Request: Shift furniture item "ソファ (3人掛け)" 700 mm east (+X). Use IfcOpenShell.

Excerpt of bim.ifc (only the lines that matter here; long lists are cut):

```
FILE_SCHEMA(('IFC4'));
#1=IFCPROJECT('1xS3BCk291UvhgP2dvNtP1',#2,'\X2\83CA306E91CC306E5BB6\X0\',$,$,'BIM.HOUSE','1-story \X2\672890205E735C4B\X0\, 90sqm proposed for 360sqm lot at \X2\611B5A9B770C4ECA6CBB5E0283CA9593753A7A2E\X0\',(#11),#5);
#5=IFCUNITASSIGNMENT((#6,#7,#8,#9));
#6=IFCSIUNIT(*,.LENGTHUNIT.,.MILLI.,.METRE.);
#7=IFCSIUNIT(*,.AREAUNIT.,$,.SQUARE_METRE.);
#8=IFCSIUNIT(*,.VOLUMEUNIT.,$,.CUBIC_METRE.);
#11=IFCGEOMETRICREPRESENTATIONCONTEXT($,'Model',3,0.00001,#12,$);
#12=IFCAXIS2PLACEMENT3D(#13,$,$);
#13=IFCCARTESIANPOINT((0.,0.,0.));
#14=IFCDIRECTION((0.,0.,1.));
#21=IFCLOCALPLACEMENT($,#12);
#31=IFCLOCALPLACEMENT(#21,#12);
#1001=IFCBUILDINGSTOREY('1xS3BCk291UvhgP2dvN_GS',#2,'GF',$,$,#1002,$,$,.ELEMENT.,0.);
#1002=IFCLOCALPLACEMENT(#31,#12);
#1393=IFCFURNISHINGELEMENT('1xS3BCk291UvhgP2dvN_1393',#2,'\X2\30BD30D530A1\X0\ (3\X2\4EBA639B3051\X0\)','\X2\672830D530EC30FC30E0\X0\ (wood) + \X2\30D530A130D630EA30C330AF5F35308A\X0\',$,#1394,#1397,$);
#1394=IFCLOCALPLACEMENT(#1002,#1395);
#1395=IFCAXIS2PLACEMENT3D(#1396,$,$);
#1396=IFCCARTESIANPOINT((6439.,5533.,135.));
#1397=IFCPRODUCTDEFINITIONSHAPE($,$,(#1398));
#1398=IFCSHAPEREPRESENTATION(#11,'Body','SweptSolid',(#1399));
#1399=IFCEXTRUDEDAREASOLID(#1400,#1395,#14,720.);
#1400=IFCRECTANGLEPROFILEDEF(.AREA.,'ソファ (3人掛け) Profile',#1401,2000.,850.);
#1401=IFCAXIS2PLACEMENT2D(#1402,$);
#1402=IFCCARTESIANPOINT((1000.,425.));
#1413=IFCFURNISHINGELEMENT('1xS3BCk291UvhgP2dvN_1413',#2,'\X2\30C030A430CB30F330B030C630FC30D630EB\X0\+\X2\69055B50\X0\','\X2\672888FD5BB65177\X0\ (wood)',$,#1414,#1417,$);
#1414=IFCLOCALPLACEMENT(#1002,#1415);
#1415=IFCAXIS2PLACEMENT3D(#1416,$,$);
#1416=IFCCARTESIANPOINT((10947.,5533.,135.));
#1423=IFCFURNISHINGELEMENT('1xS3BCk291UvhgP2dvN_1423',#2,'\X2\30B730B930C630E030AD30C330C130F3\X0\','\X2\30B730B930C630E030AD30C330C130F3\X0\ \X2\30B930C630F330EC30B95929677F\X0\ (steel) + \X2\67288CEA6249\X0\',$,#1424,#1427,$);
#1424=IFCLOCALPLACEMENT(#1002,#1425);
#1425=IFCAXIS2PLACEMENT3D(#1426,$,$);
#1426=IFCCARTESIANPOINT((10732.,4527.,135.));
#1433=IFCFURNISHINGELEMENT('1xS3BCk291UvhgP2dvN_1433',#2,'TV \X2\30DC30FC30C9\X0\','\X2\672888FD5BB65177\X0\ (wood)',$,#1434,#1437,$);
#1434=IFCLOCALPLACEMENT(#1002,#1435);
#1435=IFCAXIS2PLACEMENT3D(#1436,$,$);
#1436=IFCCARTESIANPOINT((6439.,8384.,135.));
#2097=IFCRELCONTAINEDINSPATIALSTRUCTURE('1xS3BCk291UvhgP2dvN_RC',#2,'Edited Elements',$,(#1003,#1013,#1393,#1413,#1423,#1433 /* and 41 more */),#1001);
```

```python
import ifcopenshell
import ifcopenshell.api.geometry
import ifcopenshell.util.placement
import ifcopenshell.util.unit

model = ifcopenshell.open("bim.ifc")
unit_scale = ifcopenshell.util.unit.calculate_unit_scale(model)

item = model.by_id(1393)
matrix = ifcopenshell.util.placement.get_local_placement(item.ObjectPlacement)
matrix[0, 3] += 0.7 / unit_scale
ifcopenshell.api.geometry.edit_object_placement(model, product=item, matrix=matrix, is_si=False)

print(ifcopenshell.util.placement.get_local_placement(item.ObjectPlacement).round(3) + 0.0)

model.write("bim_rev.ifc")
```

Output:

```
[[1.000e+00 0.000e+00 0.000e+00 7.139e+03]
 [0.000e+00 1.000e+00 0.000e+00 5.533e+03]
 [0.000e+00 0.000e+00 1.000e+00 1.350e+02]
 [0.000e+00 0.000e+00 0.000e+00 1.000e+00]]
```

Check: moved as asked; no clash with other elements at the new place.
